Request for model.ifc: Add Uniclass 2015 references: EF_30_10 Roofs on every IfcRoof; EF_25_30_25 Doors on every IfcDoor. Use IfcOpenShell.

First a look at what the model holds.

```python
import ifcopenshell

model = ifcopenshell.open("model.ifc")
print(model.schema)
print("classifications:", [c.Name for c in model.by_type("IfcClassification")])
for ifc_class in ("IfcDoor", "IfcRoof", "IfcStair", "IfcWall", "IfcWindow"):
    print(ifc_class, len(model.by_type(ifc_class)))
```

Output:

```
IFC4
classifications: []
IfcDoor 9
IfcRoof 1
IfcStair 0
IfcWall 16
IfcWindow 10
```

```python
import ifcopenshell
import ifcopenshell.api.classification

model = ifcopenshell.open("model.ifc")

system = ifcopenshell.api.classification.add_classification(model, classification="Uniclass 2015")

codes = {
    "IfcRoof": ("EF_30_10", "Roofs"),
    "IfcDoor": ("EF_25_30_25", "Doors"),
}
for ifc_class, (code, name) in codes.items():
    products = model.by_type(ifc_class)
    ifcopenshell.api.classification.add_reference(
        model, products=products, classification=system, identification=code, name=name
    )
    print(code, len(products))

model.write("model_edited.ifc")
```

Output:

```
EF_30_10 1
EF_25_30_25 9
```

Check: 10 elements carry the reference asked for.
